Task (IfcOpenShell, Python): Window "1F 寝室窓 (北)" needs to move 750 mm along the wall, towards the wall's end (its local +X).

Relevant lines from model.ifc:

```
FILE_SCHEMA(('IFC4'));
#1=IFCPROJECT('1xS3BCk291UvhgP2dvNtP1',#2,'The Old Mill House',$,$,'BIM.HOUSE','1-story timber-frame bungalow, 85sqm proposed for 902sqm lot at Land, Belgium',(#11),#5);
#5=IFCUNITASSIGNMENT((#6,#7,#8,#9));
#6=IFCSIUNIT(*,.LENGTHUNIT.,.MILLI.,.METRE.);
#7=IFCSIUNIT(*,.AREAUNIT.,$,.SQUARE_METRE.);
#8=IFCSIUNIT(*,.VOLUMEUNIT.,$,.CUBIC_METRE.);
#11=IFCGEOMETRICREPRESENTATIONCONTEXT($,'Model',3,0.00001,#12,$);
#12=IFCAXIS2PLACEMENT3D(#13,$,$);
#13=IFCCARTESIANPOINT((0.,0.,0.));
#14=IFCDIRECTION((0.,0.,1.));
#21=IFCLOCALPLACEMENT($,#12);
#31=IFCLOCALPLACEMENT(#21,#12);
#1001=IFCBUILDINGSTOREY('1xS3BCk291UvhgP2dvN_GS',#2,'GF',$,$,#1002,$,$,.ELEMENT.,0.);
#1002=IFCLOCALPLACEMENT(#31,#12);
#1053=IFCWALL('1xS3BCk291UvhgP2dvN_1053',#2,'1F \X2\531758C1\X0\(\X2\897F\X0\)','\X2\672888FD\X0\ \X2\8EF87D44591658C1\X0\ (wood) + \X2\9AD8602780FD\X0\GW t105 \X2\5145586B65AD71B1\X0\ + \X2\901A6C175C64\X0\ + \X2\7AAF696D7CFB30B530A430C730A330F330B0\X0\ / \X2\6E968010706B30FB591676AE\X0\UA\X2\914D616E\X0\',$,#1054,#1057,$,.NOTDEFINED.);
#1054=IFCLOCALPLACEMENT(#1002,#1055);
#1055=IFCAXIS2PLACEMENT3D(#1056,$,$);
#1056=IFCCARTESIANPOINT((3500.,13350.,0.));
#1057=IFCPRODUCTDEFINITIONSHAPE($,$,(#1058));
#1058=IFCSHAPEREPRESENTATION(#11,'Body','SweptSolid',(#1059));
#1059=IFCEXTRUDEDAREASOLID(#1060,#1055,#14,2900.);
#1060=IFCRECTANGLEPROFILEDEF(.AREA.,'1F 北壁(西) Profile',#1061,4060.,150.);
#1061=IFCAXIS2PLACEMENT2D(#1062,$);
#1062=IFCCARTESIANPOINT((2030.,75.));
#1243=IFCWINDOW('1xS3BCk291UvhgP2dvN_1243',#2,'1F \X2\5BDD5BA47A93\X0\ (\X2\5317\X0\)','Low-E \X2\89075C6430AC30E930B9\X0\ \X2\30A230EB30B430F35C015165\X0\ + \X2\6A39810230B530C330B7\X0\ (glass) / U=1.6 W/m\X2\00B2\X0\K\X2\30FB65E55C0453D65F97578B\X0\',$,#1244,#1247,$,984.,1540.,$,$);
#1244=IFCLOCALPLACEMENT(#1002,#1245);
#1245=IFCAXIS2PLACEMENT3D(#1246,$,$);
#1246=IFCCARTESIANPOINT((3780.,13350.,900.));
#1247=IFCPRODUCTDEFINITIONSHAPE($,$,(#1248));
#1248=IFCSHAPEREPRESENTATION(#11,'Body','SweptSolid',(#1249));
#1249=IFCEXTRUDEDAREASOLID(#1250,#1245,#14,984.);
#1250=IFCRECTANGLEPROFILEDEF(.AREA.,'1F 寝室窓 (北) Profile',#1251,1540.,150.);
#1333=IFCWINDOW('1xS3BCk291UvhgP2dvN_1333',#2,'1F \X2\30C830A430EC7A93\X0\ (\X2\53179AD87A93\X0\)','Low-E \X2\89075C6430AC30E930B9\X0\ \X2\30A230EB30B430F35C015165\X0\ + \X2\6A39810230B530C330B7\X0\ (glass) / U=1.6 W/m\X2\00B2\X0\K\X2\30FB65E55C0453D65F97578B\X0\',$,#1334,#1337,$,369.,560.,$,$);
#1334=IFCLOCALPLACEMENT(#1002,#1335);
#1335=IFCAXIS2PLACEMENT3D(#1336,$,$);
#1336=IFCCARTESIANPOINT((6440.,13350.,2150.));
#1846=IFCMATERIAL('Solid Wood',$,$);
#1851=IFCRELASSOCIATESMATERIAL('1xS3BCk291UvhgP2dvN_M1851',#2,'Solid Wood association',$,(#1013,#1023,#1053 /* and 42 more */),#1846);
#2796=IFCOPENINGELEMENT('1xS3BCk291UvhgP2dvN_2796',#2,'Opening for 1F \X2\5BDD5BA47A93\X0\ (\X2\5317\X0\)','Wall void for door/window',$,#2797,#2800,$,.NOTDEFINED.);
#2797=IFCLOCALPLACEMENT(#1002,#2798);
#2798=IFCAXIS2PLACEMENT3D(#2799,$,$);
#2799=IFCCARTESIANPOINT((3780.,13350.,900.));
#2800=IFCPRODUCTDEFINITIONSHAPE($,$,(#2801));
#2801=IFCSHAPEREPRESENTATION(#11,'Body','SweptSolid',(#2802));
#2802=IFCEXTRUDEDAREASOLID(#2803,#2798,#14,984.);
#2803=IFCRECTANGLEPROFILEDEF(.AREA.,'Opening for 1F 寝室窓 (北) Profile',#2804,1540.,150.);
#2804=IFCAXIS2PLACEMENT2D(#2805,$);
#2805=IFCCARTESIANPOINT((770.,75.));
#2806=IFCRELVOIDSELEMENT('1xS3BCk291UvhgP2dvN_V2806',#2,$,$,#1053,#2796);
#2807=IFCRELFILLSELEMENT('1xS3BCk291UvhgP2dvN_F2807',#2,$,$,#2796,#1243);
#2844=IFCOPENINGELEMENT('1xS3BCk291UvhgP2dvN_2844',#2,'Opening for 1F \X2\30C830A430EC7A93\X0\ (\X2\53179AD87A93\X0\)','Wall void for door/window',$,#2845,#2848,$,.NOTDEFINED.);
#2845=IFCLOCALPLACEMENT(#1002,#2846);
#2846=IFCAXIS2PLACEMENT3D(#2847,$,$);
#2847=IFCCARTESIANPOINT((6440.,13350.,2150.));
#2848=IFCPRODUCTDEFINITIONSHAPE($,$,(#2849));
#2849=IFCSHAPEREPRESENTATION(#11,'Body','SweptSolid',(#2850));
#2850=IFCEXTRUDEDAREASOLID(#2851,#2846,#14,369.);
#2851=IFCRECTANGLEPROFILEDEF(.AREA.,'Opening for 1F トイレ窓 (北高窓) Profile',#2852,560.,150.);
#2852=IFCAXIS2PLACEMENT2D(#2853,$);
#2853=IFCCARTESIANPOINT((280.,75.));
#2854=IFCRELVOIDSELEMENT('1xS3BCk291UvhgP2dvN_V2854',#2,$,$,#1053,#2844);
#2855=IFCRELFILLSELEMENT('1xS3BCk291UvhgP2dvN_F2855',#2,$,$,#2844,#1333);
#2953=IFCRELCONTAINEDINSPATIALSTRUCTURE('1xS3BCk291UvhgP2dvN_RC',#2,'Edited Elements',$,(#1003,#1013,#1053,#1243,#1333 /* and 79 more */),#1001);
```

```python
import ifcopenshell
import ifcopenshell.api.geometry
import ifcopenshell.util.placement

model = ifcopenshell.open("model.ifc")

window = model.by_guid("1xS3BCk291UvhgP2dvN_1243")
opening = window.FillsVoids[0].RelatingOpeningElement
wall = opening.VoidsElements[0].RelatingBuildingElement

wall_matrix = ifcopenshell.util.placement.get_local_placement(wall.ObjectPlacement)
shift = wall_matrix[:3, 0] * 750.0
before = ifcopenshell.util.placement.get_local_placement(window.ObjectPlacement)[:3, 3].copy()

# The window is not placed relative to its opening, so move both.
for product in (opening, window):
    matrix = ifcopenshell.util.placement.get_local_placement(product.ObjectPlacement)
    matrix[:3, 3] += shift
    ifcopenshell.api.geometry.edit_object_placement(model, product=product, matrix=matrix, is_si=False)

after = ifcopenshell.util.placement.get_local_placement(window.ObjectPlacement)[:3, 3]
print("window moved by", (after - before).round(3) + 0.0)

model.write("model_updated.ifc")
```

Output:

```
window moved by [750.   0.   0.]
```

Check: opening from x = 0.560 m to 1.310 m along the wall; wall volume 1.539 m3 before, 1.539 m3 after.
